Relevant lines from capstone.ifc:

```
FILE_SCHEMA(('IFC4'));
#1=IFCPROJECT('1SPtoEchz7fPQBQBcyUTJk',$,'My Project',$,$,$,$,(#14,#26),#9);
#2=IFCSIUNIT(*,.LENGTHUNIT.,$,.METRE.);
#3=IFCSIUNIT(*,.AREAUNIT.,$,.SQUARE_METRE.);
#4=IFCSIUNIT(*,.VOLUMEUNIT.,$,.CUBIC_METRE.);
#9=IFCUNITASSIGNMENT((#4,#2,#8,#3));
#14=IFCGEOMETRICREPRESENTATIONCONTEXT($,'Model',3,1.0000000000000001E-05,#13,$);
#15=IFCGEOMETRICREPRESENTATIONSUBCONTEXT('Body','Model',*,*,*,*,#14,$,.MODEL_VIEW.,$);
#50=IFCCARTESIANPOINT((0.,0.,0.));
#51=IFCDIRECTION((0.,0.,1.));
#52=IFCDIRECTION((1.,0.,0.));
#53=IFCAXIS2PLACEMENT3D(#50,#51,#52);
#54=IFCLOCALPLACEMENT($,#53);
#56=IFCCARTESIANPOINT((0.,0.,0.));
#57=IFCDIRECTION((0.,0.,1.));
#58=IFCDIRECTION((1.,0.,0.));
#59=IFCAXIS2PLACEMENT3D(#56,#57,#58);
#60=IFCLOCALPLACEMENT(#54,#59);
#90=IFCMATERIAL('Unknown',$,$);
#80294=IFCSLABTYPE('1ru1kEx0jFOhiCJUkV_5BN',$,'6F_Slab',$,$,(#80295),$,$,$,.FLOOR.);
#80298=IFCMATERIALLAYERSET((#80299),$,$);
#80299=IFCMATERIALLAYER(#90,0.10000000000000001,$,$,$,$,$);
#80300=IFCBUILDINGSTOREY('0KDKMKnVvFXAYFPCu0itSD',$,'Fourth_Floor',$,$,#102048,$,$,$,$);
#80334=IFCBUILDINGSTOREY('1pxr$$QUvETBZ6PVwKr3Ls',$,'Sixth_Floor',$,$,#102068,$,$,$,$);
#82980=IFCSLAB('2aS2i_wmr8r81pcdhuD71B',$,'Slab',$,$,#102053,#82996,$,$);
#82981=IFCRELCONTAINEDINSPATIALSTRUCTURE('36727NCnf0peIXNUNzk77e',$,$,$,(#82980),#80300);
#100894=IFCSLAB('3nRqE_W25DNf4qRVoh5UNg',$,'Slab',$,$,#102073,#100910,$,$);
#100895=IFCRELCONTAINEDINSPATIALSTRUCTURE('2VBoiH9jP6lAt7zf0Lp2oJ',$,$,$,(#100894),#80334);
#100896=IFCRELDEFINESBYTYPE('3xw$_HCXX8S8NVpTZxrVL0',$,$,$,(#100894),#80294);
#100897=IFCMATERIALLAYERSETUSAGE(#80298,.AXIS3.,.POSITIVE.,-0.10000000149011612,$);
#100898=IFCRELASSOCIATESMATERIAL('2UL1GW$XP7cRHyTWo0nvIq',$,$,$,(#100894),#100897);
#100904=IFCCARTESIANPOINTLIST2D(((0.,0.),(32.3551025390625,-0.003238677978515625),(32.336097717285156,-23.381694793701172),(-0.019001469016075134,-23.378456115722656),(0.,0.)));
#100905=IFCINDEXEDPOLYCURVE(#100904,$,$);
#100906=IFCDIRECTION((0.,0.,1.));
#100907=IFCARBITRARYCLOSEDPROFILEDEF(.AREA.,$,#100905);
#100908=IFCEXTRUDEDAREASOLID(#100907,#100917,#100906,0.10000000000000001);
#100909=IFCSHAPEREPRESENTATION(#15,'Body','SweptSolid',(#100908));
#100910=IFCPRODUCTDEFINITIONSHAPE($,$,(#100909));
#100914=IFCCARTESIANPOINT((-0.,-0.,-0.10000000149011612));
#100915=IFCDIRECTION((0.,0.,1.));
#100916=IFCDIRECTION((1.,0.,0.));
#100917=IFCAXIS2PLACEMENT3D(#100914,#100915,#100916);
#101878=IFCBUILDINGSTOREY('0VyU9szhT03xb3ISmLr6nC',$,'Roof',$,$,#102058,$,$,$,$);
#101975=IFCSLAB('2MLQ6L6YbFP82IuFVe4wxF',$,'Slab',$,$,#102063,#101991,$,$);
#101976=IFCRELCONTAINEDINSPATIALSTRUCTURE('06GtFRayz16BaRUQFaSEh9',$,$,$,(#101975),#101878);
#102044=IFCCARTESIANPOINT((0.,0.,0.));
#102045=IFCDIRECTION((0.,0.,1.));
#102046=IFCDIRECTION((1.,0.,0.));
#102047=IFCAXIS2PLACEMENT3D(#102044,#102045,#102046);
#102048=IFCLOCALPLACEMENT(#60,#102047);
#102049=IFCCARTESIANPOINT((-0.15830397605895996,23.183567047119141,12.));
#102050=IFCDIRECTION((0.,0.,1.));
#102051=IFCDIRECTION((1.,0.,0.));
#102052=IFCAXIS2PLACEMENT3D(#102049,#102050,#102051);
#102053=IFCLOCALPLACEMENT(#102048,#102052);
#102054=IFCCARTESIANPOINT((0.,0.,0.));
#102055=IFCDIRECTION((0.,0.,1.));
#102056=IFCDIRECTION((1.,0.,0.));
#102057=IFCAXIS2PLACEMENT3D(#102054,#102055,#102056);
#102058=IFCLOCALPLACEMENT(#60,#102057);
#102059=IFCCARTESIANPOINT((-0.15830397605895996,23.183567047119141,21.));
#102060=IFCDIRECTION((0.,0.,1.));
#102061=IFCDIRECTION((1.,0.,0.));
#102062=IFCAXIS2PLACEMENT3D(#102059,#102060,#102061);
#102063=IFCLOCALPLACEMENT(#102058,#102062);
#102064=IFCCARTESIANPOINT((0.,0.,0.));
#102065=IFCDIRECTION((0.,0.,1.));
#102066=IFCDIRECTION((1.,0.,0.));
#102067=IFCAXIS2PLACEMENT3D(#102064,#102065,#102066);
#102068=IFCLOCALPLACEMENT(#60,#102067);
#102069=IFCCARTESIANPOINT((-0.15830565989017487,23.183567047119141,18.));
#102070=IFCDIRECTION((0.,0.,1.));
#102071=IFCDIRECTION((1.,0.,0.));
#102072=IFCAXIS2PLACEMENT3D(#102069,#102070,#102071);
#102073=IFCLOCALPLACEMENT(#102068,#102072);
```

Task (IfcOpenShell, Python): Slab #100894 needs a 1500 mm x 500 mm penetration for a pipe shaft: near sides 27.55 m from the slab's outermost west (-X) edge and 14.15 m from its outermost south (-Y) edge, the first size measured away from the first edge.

```python
import numpy as np
import ifcopenshell
import ifcopenshell.api.feature
import ifcopenshell.api.geometry
import ifcopenshell.api.root
import ifcopenshell.geom
import ifcopenshell.util.placement
import ifcopenshell.util.representation
import ifcopenshell.util.shape
import ifcopenshell.util.unit

model = ifcopenshell.open("capstone.ifc")
unit_scale = ifcopenshell.util.unit.calculate_unit_scale(model)
settings = ifcopenshell.geom.settings()


def volume(element):
    """Net volume in cubic metres, openings subtracted."""
    shape = ifcopenshell.geom.create_shape(settings, element)
    return ifcopenshell.util.shape.get_volume(shape.geometry)


slab = model.by_guid("3nRqE_W25DNf4qRVoh5UNg")
before = volume(slab)

# Extent in the slab's own axes, in metres. The edges named are its -X and -Y sides.
slab_shape = ifcopenshell.geom.create_shape(settings, slab)
vertices = ifcopenshell.util.shape.get_vertices(slab_shape.geometry)
x_min, y_min, bottom = vertices.min(axis=0)
top = vertices[:, 2].max()

opening = ifcopenshell.api.root.create_entity(model, ifc_class="IfcOpeningElement", name="Pipe shaft opening", predefined_type="OPENING")
context = ifcopenshell.util.representation.get_context(model, "Model", "Body", "MODEL_VIEW")
width, depth = 1.5, 0.5
outline = [(0.0, 0.0), (width, 0.0), (width, depth), (0.0, depth), (0.0, 0.0)]
# Overshoot both faces by 50 mm so the cut is clean.
shape = ifcopenshell.api.geometry.add_slab_representation(
    model, context=context, depth=top - bottom + 0.1, polyline=outline
)
ifcopenshell.api.geometry.assign_representation(model, product=opening, representation=shape)

matrix = ifcopenshell.util.placement.get_local_placement(slab.ObjectPlacement)
matrix[:, 3] = matrix @ np.append(np.array([x_min + 27.55, y_min + 14.15, bottom - 0.05]) / unit_scale, 1.0)
ifcopenshell.api.geometry.edit_object_placement(model, product=opening, matrix=matrix, is_si=False)
ifcopenshell.api.feature.add_feature(model, feature=opening, element=slab)

after = volume(slab)

print(f"slab volume {before:.3f} -> {after:.3f} m3")

model.write("capstone-out.ifc")
```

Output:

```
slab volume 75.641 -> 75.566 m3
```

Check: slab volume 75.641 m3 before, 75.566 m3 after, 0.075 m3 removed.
